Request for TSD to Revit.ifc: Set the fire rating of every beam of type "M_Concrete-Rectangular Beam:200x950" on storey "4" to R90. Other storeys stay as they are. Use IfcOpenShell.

First a look at what the model holds.

```python
import ifcopenshell
import ifcopenshell.util.element

model = ifcopenshell.open("TSD to Revit.ifc")
print(model.schema)
storey = next(s for s in model.by_type("IfcBuildingStorey") if s.Name == "4")
beams = [e for e in ifcopenshell.util.element.get_decomposition(storey) if e.is_a("IfcBeam")]
seen = {}
for e in beams:
    element_type = ifcopenshell.util.element.get_type(e)
    key = (element_type.Name if element_type != e and element_type else None, ifcopenshell.util.element.get_pset(e, "Pset_BeamCommon", "FireRating"))
    seen[key] = seen.get(key, 0) + 1
for (name, value), count in sorted(seen.items(), key=str):
    print(count, "x", name, "|", value)
```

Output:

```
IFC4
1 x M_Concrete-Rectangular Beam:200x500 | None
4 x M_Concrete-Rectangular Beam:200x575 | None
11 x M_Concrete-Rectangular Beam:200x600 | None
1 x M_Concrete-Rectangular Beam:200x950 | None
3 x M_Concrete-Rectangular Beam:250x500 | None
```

```python
import ifcopenshell
import ifcopenshell.api.pset
import ifcopenshell.util.element

model = ifcopenshell.open("TSD to Revit.ifc")

storey = next(s for s in model.by_type("IfcBuildingStorey") if s.Name == "4")
beams = [e for e in ifcopenshell.util.element.get_decomposition(storey) if e.is_a("IfcBeam")]

count = 0
for e in beams:
    element_type = ifcopenshell.util.element.get_type(e)
    if element_type in (None, e) or element_type.Name != "M_Concrete-Rectangular Beam:200x950":
        continue
    # add_pset returns the element's existing set when there is one.
    pset = ifcopenshell.api.pset.add_pset(model, product=e, name="Pset_BeamCommon")
    ifcopenshell.api.pset.edit_pset(model, pset=pset, properties={"FireRating": "R90"})
    count += 1

print(count, "beams updated")

model.write("TSD to Revit-out.ifc")
```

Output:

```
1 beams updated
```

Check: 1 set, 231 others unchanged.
